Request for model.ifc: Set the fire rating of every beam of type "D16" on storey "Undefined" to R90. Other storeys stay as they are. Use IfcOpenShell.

First a look at what the model holds.

```python
import ifcopenshell
import ifcopenshell.util.element

model = ifcopenshell.open("model.ifc")
print(model.schema)
storey = next(s for s in model.by_type("IfcBuildingStorey") if s.Name == "Undefined")
beams = [e for e in ifcopenshell.util.element.get_decomposition(storey) if e.is_a("IfcBeam")]
seen = {}
for e in beams:
    element_type = ifcopenshell.util.element.get_type(e)
    key = (element_type.Name if element_type != e and element_type else None, ifcopenshell.util.element.get_pset(e, "Pset_BeamCommon", "FireRating"))
    seen[key] = seen.get(key, 0) + 1
for (name, value), count in sorted(seen.items(), key=str):
    print(count, "x", name, "|", value)
```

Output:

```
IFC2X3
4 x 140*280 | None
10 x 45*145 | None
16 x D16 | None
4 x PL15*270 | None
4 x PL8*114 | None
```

```python
import ifcopenshell
import ifcopenshell.api.pset
import ifcopenshell.util.element

model = ifcopenshell.open("model.ifc")

storey = next(s for s in model.by_type("IfcBuildingStorey") if s.Name == "Undefined")
beams = [e for e in ifcopenshell.util.element.get_decomposition(storey) if e.is_a("IfcBeam")]

count = 0
for e in beams:
    element_type = ifcopenshell.util.element.get_type(e)
    if element_type in (None, e) or element_type.Name != "D16":
        continue
    # add_pset returns the element's existing set when there is one.
    pset = ifcopenshell.api.pset.add_pset(model, product=e, name="Pset_BeamCommon")
    ifcopenshell.api.pset.edit_pset(model, pset=pset, properties={"FireRating": "R90"})
    count += 1

print(count, "beams updated")

model.write("model_rev.ifc")
```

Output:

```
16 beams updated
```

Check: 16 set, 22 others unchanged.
